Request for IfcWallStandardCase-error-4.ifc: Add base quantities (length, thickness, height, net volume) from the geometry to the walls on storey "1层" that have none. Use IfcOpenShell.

First a look at what the model holds.

```python
import ifcopenshell
import ifcopenshell.util.element
import ifcopenshell.util.unit

model = ifcopenshell.open("IfcWallStandardCase-error-4.ifc")
print(model.schema)
for unit_type in ("LENGTHUNIT", "AREAUNIT", "VOLUMEUNIT"):
    print(unit_type, ifcopenshell.util.unit.calculate_unit_scale(model, unit_type))
storey = next(s for s in model.by_type("IfcBuildingStorey") if s.Name == "1层")
walls = [e for e in ifcopenshell.util.element.get_decomposition(storey) if e.is_a("IfcWall")]
for e in sorted(walls, key=lambda e: e.id()):
    print(e.id(), e.is_a(), e.Name, list(ifcopenshell.util.element.get_psets(e, qtos_only=True)), sep=" | ")
```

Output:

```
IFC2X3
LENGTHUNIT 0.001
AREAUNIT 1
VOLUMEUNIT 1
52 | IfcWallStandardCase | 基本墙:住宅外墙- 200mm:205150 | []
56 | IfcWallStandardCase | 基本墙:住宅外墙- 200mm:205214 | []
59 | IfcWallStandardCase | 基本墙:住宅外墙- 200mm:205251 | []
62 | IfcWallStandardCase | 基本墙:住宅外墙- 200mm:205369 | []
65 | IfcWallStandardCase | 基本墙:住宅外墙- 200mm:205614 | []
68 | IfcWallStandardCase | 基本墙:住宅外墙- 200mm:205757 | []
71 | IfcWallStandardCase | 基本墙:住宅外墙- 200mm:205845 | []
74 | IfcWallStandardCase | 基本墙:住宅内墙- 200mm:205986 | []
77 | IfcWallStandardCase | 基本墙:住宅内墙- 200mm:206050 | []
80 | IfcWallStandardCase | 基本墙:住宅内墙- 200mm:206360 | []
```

```python
import ifcopenshell
import ifcopenshell.api.pset
import ifcopenshell.geom
import ifcopenshell.util.element
import ifcopenshell.util.shape
import ifcopenshell.util.unit

model = ifcopenshell.open("IfcWallStandardCase-error-4.ifc")
unit_scale = ifcopenshell.util.unit.calculate_unit_scale(model)
volume_scale = ifcopenshell.util.unit.calculate_unit_scale(model, "VOLUMEUNIT")
settings = ifcopenshell.geom.settings()

storey = next(s for s in model.by_type("IfcBuildingStorey") if s.Name == "1层")
walls = [e for e in ifcopenshell.util.element.get_decomposition(storey) if e.is_a("IfcWall")]

for e in sorted(walls, key=lambda e: e.id()):
    if ifcopenshell.util.element.get_psets(e, qtos_only=True, should_inherit=False):
        continue
    # Geometry comes back in metres, in the element's own axes.
    shape = ifcopenshell.geom.create_shape(settings, e)
    values = {
        "Length": ifcopenshell.util.shape.get_x(shape.geometry) / unit_scale,
        "Width": ifcopenshell.util.shape.get_y(shape.geometry) / unit_scale,
        "Height": ifcopenshell.util.shape.get_z(shape.geometry) / unit_scale,
        "NetVolume": ifcopenshell.util.shape.get_volume(shape.geometry) / volume_scale,
    }
    qto = ifcopenshell.api.pset.add_qto(model, product=e, name="BaseQuantities")
    ifcopenshell.api.pset.edit_qto(model, qto=qto, properties=values)
    print(e.id(), {k: round(v, 3) for k, v in values.items()})

model.write("IfcWallStandardCase-error-4-out.ifc")
```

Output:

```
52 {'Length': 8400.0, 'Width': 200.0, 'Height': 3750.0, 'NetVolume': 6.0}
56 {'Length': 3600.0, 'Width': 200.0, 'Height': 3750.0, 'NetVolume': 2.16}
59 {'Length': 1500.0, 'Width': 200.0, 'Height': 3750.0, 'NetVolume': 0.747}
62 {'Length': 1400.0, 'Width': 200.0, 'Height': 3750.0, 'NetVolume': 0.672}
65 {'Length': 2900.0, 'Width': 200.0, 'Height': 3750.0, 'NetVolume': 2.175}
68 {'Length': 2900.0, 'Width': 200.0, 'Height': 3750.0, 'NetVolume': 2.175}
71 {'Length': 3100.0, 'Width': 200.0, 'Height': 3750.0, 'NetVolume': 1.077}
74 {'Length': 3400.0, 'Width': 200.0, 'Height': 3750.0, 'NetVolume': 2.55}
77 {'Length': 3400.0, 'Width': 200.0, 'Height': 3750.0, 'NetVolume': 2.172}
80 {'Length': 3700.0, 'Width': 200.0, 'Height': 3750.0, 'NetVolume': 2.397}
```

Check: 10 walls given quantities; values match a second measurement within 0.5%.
